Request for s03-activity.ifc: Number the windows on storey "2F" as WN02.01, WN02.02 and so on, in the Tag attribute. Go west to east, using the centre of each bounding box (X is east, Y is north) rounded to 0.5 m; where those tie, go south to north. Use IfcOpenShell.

First a look at what the model holds.

```python
import ifcopenshell
import ifcopenshell.util.element
import ifcopenshell.util.placement

model = ifcopenshell.open("s03-activity.ifc")
print(model.schema)
storey = next(s for s in model.by_type("IfcBuildingStorey") if s.Name == "2F")
windows = [e for e in ifcopenshell.util.element.get_decomposition(storey) if e.is_a("IfcWindow")]
for e in sorted(windows, key=lambda e: e.id()):
    origin = ifcopenshell.util.placement.get_local_placement(e.ObjectPlacement)[:3, 3]
    print(e.id(), e.Tag, e.Name, origin.round(2) + 0.0, sep=" | ")
```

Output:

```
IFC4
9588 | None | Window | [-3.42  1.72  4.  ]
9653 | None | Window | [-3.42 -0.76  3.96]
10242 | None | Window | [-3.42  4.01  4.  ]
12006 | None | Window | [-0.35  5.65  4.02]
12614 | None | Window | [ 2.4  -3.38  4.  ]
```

```python
import ifcopenshell
import ifcopenshell.geom
import ifcopenshell.util.element
import ifcopenshell.util.shape

model = ifcopenshell.open("s03-activity.ifc")
settings = ifcopenshell.geom.settings()
settings.set("use-world-coords", True)


def centre(element):
    shape = ifcopenshell.geom.create_shape(settings, element)
    return ifcopenshell.util.shape.get_bbox_centroid(shape.geometry)


storey = next(s for s in model.by_type("IfcBuildingStorey") if s.Name == "2F")
windows = [e for e in ifcopenshell.util.element.get_decomposition(storey) if e.is_a("IfcWindow")]

# Insertion points can sit at a corner or the storey origin, so sort by the geometry (in metres).
centres = {e: centre(e) for e in windows}
windows.sort(key=lambda e: (round(centres[e][0] / 0.5), centres[e][1]))

for i, e in enumerate(windows, start=1):
    number = f"WN02.{i:02d}"
    e.Tag = number
    print(e.id(), number)

model.write("s03-activity-out.ifc")
```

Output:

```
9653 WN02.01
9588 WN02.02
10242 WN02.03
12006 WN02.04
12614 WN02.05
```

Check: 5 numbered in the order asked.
